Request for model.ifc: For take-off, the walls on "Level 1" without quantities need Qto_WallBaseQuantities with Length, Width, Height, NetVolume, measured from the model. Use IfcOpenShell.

First a look at what the model holds.

```python
import ifcopenshell
import ifcopenshell.util.element
import ifcopenshell.util.unit

model = ifcopenshell.open("model.ifc")
print(model.schema)
for unit_type in ("LENGTHUNIT", "AREAUNIT", "VOLUMEUNIT"):
    print(unit_type, ifcopenshell.util.unit.calculate_unit_scale(model, unit_type))
storey = next(s for s in model.by_type("IfcBuildingStorey") if s.Name == "Level 1")
walls = [e for e in ifcopenshell.util.element.get_decomposition(storey) if e.is_a("IfcWall")]
for e in sorted(walls, key=lambda e: e.id()):
    print(e.id(), e.is_a(), e.Name, list(ifcopenshell.util.element.get_psets(e, qtos_only=True)), sep=" | ")
```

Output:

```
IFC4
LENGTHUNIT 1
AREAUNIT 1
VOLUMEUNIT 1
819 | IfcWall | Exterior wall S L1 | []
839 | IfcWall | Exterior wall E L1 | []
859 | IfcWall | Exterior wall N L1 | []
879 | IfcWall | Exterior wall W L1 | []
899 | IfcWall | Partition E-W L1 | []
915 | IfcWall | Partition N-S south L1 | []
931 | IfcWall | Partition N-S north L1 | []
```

```python
import ifcopenshell
import ifcopenshell.api.pset
import ifcopenshell.geom
import ifcopenshell.util.element
import ifcopenshell.util.shape
import ifcopenshell.util.unit

model = ifcopenshell.open("model.ifc")
unit_scale = ifcopenshell.util.unit.calculate_unit_scale(model)
volume_scale = ifcopenshell.util.unit.calculate_unit_scale(model, "VOLUMEUNIT")
settings = ifcopenshell.geom.settings()

storey = next(s for s in model.by_type("IfcBuildingStorey") if s.Name == "Level 1")
walls = [e for e in ifcopenshell.util.element.get_decomposition(storey) if e.is_a("IfcWall")]

for e in sorted(walls, key=lambda e: e.id()):
    if ifcopenshell.util.element.get_psets(e, qtos_only=True, should_inherit=False):
        continue
    # Geometry comes back in metres, in the element's own axes.
    shape = ifcopenshell.geom.create_shape(settings, e)
    values = {
        "Length": ifcopenshell.util.shape.get_x(shape.geometry) / unit_scale,
        "Width": ifcopenshell.util.shape.get_y(shape.geometry) / unit_scale,
        "Height": ifcopenshell.util.shape.get_z(shape.geometry) / unit_scale,
        "NetVolume": ifcopenshell.util.shape.get_volume(shape.geometry) / volume_scale,
    }
    qto = ifcopenshell.api.pset.add_qto(model, product=e, name="Qto_WallBaseQuantities")
    ifcopenshell.api.pset.edit_qto(model, qto=qto, properties=values)
    print(e.id(), {k: round(v, 3) for k, v in values.items()})

model.write("model-out.ifc")
```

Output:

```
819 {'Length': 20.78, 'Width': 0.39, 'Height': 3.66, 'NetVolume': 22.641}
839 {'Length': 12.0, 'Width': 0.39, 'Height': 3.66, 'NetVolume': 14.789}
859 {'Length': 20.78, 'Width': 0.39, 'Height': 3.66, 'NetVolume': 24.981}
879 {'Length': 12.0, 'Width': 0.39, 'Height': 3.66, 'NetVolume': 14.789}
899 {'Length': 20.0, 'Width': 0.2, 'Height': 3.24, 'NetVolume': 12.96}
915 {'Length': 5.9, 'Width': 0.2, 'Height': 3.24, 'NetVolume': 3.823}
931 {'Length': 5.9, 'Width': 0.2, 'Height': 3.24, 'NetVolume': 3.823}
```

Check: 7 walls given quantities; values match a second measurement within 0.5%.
